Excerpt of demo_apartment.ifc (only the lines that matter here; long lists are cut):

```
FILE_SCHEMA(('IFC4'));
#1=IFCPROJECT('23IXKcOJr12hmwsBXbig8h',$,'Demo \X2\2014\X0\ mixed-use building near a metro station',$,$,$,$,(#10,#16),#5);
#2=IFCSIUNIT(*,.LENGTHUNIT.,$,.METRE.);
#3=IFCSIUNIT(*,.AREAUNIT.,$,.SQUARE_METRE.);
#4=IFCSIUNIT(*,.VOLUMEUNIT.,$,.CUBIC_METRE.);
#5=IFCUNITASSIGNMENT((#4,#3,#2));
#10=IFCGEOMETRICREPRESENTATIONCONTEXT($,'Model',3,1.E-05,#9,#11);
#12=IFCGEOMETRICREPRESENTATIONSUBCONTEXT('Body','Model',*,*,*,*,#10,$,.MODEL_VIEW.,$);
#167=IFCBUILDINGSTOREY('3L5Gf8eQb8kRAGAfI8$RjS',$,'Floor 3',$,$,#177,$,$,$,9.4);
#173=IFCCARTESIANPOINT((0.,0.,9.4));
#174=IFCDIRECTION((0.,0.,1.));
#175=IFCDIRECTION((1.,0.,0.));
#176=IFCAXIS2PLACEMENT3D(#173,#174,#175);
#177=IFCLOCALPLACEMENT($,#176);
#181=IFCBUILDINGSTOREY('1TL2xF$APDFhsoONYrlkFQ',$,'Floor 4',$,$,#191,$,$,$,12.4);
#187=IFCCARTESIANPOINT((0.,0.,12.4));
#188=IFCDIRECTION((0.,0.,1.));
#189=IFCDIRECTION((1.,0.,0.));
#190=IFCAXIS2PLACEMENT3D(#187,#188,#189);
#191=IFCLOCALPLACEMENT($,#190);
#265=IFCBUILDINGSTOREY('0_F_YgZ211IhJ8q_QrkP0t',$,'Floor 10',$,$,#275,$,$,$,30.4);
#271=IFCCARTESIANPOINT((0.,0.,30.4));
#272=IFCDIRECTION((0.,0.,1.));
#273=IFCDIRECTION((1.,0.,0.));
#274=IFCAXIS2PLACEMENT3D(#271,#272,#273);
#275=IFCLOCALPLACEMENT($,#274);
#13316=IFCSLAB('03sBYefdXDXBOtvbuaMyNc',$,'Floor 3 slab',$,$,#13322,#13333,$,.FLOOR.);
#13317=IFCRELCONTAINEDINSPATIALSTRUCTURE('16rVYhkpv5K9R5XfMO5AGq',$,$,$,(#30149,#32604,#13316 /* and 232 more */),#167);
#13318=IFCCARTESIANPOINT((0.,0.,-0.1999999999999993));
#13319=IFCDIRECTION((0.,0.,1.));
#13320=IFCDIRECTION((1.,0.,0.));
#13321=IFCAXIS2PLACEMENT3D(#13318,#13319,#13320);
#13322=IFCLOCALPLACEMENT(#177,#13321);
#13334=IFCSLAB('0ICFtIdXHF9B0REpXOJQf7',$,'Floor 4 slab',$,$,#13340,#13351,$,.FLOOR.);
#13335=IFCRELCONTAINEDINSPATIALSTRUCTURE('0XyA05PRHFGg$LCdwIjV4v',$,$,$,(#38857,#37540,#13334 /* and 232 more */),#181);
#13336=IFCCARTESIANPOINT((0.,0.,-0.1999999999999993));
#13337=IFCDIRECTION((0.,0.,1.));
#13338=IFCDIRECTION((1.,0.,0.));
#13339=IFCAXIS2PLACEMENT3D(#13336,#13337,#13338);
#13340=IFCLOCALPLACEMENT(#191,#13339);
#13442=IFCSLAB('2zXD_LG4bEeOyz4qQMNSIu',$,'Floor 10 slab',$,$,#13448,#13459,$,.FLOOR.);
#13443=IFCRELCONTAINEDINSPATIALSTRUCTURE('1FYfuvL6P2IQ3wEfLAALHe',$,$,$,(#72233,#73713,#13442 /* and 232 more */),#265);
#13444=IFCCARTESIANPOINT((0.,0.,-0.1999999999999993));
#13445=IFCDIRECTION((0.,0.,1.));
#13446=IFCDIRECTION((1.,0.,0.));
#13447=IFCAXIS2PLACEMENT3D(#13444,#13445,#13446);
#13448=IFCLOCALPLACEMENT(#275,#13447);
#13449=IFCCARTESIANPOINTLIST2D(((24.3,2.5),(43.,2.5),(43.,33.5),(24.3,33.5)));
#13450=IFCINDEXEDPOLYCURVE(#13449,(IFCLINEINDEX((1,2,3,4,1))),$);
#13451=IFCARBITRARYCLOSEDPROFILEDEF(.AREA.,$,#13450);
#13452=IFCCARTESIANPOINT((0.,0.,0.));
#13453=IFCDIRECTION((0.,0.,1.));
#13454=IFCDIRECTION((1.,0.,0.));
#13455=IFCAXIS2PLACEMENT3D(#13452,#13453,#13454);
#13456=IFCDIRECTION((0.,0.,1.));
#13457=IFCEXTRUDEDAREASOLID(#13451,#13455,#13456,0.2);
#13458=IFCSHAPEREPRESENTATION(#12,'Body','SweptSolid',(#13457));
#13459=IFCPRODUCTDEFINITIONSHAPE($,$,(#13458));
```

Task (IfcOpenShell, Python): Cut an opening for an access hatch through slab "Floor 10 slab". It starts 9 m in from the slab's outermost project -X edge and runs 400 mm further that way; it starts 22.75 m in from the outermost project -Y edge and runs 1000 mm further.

```python
import numpy as np
import ifcopenshell
import ifcopenshell.api.feature
import ifcopenshell.api.geometry
import ifcopenshell.api.root
import ifcopenshell.geom
import ifcopenshell.util.placement
import ifcopenshell.util.representation
import ifcopenshell.util.shape
import ifcopenshell.util.unit

model = ifcopenshell.open("demo_apartment.ifc")
unit_scale = ifcopenshell.util.unit.calculate_unit_scale(model)
settings = ifcopenshell.geom.settings()


def volume(element):
    """Net volume in cubic metres, openings subtracted."""
    shape = ifcopenshell.geom.create_shape(settings, element)
    return ifcopenshell.util.shape.get_volume(shape.geometry)


slab = model.by_guid("2zXD_LG4bEeOyz4qQMNSIu")
before = volume(slab)

# Extent in the slab's own axes, in metres. The edges named are its -X and -Y sides.
slab_shape = ifcopenshell.geom.create_shape(settings, slab)
vertices = ifcopenshell.util.shape.get_vertices(slab_shape.geometry)
x_min, y_min, bottom = vertices.min(axis=0)
top = vertices[:, 2].max()

opening = ifcopenshell.api.root.create_entity(model, ifc_class="IfcOpeningElement", name="Access hatch opening", predefined_type="OPENING")
context = ifcopenshell.util.representation.get_context(model, "Model", "Body", "MODEL_VIEW")
width, depth = 0.4, 1
outline = [(0.0, 0.0), (width, 0.0), (width, depth), (0.0, depth), (0.0, 0.0)]
# Overshoot both faces by 50 mm so the cut is clean.
shape = ifcopenshell.api.geometry.add_slab_representation(
    model, context=context, depth=top - bottom + 0.1, polyline=outline
)
ifcopenshell.api.geometry.assign_representation(model, product=opening, representation=shape)

matrix = ifcopenshell.util.placement.get_local_placement(slab.ObjectPlacement)
matrix[:, 3] = matrix @ np.append(np.array([x_min + 9, y_min + 22.75, bottom - 0.05]) / unit_scale, 1.0)
ifcopenshell.api.geometry.edit_object_placement(model, product=opening, matrix=matrix, is_si=False)
ifcopenshell.api.feature.add_feature(model, feature=opening, element=slab)

after = volume(slab)

print(f"slab volume {before:.3f} -> {after:.3f} m3")

model.write("demo_apartment-out.ifc")
```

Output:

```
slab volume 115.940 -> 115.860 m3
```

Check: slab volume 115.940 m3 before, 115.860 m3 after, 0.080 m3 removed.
